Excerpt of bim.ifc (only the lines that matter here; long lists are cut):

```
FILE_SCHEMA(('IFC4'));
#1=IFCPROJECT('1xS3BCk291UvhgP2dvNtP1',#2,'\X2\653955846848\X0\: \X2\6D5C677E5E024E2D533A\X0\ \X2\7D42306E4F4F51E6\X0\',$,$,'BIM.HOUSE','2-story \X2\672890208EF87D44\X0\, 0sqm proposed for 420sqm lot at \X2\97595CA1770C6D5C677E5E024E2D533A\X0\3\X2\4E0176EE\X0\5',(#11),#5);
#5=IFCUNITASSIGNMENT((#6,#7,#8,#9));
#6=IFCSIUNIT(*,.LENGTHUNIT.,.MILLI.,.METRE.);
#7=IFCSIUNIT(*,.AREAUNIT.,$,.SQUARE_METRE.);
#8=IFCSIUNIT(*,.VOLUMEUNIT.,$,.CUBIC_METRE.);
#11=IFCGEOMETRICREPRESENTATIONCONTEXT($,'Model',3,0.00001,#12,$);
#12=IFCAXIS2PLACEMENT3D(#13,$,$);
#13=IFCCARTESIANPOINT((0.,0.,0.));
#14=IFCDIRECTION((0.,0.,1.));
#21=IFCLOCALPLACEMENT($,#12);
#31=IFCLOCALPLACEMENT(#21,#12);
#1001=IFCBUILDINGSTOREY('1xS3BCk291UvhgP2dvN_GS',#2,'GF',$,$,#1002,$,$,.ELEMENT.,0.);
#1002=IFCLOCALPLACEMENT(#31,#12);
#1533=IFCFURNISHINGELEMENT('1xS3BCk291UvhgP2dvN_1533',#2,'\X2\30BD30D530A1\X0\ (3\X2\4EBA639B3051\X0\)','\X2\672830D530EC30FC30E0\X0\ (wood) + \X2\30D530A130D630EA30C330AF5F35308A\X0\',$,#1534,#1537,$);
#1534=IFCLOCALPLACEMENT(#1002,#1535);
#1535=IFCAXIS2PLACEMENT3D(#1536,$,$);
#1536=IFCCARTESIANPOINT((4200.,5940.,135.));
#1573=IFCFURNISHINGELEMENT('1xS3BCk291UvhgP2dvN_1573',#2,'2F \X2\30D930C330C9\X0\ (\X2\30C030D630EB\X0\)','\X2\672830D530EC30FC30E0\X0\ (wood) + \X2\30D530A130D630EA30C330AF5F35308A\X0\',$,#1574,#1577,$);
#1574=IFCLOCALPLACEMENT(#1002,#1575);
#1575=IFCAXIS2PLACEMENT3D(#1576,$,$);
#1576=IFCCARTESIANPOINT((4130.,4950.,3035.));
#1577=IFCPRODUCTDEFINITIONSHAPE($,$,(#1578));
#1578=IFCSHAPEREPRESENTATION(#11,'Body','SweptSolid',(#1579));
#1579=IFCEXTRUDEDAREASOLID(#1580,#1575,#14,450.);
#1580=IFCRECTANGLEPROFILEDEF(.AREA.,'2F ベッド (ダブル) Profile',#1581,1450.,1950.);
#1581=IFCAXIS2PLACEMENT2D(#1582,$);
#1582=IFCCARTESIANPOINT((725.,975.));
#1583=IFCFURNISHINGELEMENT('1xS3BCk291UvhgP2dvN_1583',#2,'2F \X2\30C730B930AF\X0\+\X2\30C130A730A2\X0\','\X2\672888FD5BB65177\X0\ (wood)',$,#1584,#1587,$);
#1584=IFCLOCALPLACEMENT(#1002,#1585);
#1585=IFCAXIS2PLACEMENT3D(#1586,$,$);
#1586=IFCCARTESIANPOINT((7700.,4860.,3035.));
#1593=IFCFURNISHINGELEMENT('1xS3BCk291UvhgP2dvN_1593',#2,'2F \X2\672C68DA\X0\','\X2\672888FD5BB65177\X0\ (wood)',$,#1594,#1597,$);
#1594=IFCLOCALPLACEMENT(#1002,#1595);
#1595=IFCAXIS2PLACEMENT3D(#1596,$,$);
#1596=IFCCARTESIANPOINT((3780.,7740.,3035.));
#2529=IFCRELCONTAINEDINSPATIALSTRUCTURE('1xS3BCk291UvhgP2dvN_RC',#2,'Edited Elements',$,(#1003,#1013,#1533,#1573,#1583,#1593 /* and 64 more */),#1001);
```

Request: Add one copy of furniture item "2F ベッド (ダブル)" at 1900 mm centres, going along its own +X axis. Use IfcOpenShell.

```python
import ifcopenshell
import ifcopenshell.api.geometry
import ifcopenshell.api.root
import ifcopenshell.util.element
import ifcopenshell.util.placement
import ifcopenshell.util.unit

model = ifcopenshell.open("bim.ifc")
unit_scale = ifcopenshell.util.unit.calculate_unit_scale(model)


def reuse_history(source, copy):
    """copy_class also copies each property set's owner history, people and application; keep the originals."""
    for rel in copy.IsDefinedBy:
        if rel.is_a("IfcRelDefinesByProperties") and (history := rel.RelatingPropertyDefinition.OwnerHistory):
            rel.RelatingPropertyDefinition.OwnerHistory = source.OwnerHistory
            ifcopenshell.util.element.remove_deep2(model, history)


source = model.by_guid("1xS3BCk291UvhgP2dvN_1573")
base = ifcopenshell.util.placement.get_local_placement(source.ObjectPlacement)
step = base[:3, 0] * 1.9 / unit_scale

for i in range(1, 2):
    copy = ifcopenshell.api.root.copy_class(model, product=source)
    copy.Representation = ifcopenshell.util.element.copy_deep(
        model, source.Representation, exclude=["IfcGeometricRepresentationContext", "IfcRepresentationMap"]
    )
    reuse_history(source, copy)
    matrix = base.copy()
    matrix[:3, 3] += i * step
    print("added at", matrix[:3, 3].round(3) + 0.0)
    ifcopenshell.api.geometry.edit_object_placement(model, product=copy, matrix=matrix, is_si=False)

model.write("bim_updated.ifc")
```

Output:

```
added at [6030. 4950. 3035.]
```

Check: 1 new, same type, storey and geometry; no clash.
